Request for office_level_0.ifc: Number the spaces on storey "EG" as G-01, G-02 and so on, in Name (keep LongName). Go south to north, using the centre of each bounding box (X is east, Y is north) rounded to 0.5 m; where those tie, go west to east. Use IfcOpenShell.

First a look at what the model holds.

```python
import ifcopenshell
import ifcopenshell.util.element
import ifcopenshell.util.placement

model = ifcopenshell.open("office_level_0.ifc")
print(model.schema)
storey = next(s for s in model.by_type("IfcBuildingStorey") if s.Name == "EG")
spaces = [e for e in ifcopenshell.util.element.get_decomposition(storey) if e.is_a("IfcSpace")]
for e in sorted(spaces, key=lambda e: e.id()):
    origin = ifcopenshell.util.placement.get_local_placement(e.ObjectPlacement)[:3, 3]
    print(e.id(), e.Name, e.LongName, origin.round(2) + 0.0, sep=" | ")
```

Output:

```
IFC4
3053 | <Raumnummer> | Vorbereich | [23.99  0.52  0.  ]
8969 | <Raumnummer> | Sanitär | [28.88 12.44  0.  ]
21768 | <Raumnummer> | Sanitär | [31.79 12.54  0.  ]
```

```python
import ifcopenshell
import ifcopenshell.geom
import ifcopenshell.util.element
import ifcopenshell.util.shape

model = ifcopenshell.open("office_level_0.ifc")
settings = ifcopenshell.geom.settings()
settings.set("use-world-coords", True)


def centre(element):
    shape = ifcopenshell.geom.create_shape(settings, element)
    return ifcopenshell.util.shape.get_bbox_centroid(shape.geometry)


storey = next(s for s in model.by_type("IfcBuildingStorey") if s.Name == "EG")
spaces = [e for e in ifcopenshell.util.element.get_decomposition(storey) if e.is_a("IfcSpace")]

# Insertion points can sit at a corner or the storey origin, so sort by the geometry (in metres).
centres = {e: centre(e) for e in spaces}
spaces.sort(key=lambda e: (round(centres[e][1] / 0.5), centres[e][0]))

for i, e in enumerate(spaces, start=1):
    number = f"G-{i:02d}"
    e.Name = number
    print(e.id(), number)

model.write("office_level_0_updated.ifc")
```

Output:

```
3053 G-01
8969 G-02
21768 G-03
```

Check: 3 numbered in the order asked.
